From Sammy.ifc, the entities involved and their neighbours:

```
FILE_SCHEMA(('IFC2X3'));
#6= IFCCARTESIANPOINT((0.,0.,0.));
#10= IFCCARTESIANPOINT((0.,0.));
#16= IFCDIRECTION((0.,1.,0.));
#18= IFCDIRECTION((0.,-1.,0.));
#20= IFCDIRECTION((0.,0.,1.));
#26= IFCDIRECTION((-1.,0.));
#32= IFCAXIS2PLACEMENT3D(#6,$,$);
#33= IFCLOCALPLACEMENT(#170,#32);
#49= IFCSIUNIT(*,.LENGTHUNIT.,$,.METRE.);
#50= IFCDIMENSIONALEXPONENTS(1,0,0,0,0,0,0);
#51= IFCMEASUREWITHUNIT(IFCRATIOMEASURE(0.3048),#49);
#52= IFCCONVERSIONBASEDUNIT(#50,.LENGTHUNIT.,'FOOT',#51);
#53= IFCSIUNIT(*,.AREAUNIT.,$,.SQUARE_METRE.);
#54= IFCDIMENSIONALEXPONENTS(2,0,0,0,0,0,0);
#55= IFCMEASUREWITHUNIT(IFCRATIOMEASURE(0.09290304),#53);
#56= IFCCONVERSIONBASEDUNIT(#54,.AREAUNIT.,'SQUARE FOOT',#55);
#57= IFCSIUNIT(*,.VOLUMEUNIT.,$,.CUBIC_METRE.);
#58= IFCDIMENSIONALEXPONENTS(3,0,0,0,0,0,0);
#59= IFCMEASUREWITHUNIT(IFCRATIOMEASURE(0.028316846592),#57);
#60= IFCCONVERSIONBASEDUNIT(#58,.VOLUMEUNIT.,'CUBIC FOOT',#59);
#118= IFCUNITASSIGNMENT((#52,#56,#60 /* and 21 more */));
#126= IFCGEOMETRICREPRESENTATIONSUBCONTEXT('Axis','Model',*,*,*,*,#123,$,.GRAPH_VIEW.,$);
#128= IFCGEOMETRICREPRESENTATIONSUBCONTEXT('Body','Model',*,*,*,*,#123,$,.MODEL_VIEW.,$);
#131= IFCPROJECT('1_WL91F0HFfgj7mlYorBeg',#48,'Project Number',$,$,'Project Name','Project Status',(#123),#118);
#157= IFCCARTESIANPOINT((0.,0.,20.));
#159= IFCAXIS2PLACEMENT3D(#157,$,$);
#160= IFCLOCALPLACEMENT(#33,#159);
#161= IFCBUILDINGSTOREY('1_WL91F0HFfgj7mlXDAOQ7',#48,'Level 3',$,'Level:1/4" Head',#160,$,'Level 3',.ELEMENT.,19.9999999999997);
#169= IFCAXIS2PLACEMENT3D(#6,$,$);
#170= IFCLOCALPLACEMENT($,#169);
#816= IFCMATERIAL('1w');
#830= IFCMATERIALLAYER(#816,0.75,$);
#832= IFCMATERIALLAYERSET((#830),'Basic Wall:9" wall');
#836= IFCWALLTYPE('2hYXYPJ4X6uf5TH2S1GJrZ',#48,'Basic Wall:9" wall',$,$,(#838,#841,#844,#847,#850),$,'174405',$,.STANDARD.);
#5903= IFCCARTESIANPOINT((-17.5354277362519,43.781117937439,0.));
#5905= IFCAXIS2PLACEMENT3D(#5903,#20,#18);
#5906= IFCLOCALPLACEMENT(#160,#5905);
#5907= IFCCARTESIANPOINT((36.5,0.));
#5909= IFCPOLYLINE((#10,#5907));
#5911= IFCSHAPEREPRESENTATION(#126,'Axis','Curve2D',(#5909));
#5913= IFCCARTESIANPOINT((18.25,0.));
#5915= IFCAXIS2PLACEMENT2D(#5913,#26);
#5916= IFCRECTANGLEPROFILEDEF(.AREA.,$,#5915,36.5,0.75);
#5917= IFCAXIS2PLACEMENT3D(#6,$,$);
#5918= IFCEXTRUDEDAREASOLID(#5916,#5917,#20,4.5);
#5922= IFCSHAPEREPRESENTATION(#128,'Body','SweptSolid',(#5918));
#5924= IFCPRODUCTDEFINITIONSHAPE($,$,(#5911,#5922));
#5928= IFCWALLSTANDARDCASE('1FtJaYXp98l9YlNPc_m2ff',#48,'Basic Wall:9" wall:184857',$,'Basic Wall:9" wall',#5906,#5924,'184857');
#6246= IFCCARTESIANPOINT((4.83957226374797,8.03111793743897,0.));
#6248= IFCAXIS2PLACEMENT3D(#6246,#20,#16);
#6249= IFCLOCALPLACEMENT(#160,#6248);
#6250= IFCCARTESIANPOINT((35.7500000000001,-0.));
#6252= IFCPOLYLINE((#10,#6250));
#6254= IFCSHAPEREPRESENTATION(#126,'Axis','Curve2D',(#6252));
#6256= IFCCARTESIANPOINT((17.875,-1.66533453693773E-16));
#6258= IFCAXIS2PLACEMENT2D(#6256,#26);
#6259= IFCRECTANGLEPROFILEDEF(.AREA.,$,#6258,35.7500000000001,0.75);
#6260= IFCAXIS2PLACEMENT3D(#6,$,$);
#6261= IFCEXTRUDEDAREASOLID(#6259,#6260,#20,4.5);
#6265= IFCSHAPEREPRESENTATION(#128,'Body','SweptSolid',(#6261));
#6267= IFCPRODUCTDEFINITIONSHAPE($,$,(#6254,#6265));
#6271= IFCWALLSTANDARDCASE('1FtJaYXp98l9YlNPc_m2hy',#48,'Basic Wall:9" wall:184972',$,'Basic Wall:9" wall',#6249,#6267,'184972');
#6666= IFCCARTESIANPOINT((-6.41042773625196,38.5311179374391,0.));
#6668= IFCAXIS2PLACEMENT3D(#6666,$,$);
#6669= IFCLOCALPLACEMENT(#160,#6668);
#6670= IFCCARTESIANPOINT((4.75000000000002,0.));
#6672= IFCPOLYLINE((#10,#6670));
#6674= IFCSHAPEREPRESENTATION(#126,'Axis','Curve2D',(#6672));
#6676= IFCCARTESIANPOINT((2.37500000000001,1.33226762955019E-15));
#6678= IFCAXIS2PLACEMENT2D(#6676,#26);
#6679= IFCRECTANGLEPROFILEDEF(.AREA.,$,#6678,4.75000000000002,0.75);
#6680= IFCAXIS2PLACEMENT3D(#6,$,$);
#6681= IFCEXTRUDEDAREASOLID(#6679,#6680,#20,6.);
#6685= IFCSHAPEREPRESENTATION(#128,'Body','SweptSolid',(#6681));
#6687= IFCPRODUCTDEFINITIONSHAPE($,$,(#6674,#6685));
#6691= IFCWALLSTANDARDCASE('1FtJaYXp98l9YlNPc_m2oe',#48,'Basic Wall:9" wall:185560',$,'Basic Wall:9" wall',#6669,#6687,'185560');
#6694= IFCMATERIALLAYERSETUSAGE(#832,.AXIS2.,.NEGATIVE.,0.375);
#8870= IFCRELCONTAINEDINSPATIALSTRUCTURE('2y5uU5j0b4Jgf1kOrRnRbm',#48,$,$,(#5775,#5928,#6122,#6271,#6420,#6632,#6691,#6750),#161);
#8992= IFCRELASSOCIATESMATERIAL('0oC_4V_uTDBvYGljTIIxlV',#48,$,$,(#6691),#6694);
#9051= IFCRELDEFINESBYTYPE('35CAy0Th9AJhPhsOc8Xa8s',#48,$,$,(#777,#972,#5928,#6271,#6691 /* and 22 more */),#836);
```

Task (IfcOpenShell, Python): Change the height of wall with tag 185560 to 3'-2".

```python
import ifcopenshell
import ifcopenshell.geom
import ifcopenshell.util.representation
import ifcopenshell.util.shape
import ifcopenshell.util.unit

model = ifcopenshell.open("Sammy.ifc")
unit_scale = ifcopenshell.util.unit.calculate_unit_scale(model)
settings = ifcopenshell.geom.settings()


def volume(element):
    """Net volume in cubic metres, openings subtracted."""
    shape = ifcopenshell.geom.create_shape(settings, element)
    return ifcopenshell.util.shape.get_volume(shape.geometry)


wall = model.by_id(6691)
before = volume(wall)

body = ifcopenshell.util.representation.get_representation(wall, "Model", "Body")
solid = body.Items[0]
old_height = solid.Depth
solid.Depth = 38 * 0.0254 / unit_scale
after = volume(wall)

print(f"height {old_height:g} -> {solid.Depth:g}, volume {before:.3f} -> {after:.3f} m3")

model.write("Sammy_rev.ifc")
```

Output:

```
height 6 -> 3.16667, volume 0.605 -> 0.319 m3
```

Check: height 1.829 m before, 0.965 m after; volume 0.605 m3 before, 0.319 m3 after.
